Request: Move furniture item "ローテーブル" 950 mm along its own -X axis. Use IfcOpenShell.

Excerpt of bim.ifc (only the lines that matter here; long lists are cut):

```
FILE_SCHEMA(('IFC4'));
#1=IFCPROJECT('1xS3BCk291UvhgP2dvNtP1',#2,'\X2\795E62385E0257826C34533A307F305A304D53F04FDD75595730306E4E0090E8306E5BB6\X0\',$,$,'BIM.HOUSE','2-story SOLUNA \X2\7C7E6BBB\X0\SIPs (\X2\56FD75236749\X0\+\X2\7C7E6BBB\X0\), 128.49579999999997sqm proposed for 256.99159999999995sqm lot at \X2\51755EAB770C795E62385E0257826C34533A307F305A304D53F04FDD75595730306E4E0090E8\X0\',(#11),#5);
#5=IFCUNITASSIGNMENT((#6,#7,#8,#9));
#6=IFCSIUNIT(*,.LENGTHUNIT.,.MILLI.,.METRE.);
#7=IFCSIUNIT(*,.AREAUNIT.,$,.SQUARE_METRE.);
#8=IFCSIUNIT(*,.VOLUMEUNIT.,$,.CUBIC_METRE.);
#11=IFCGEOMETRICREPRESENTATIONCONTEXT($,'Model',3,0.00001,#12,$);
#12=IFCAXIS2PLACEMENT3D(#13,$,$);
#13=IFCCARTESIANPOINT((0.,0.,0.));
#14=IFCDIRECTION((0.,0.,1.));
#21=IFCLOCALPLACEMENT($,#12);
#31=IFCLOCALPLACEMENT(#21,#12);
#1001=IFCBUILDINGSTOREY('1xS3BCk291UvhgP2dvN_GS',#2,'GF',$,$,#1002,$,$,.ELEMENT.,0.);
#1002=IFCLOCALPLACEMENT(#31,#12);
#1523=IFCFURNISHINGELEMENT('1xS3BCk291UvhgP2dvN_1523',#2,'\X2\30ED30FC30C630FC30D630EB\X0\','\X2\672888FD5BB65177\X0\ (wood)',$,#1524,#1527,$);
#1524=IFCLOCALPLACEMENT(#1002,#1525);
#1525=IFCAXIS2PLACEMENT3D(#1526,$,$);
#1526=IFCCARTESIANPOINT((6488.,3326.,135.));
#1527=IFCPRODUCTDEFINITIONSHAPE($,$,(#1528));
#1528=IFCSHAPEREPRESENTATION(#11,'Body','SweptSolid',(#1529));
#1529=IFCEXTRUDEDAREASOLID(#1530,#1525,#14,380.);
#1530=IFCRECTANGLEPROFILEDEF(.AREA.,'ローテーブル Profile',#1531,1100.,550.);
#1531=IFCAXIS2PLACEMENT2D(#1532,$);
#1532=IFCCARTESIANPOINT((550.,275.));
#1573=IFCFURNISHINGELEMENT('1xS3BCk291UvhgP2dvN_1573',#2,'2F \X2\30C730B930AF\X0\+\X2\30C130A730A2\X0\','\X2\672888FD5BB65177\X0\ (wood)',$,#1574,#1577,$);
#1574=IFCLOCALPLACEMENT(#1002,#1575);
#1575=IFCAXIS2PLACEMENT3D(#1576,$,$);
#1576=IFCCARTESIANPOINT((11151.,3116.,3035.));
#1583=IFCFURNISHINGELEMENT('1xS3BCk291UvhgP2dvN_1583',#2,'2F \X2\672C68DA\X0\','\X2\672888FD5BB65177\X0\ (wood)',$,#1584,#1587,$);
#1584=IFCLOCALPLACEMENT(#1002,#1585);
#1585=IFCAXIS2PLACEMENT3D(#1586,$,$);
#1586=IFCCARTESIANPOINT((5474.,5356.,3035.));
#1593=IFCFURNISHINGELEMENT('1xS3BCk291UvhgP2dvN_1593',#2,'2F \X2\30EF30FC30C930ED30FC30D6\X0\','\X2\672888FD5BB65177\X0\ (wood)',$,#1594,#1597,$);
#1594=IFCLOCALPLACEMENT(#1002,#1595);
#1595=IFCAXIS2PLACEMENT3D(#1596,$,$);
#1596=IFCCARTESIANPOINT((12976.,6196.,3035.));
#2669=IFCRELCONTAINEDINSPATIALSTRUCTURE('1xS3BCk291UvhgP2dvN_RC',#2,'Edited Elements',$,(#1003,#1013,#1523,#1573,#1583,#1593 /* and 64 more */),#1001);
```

```python
import ifcopenshell
import ifcopenshell.api.geometry
import ifcopenshell.util.placement

model = ifcopenshell.open("bim.ifc")

item = model.by_guid("1xS3BCk291UvhgP2dvN_1523")
matrix = ifcopenshell.util.placement.get_local_placement(item.ObjectPlacement)
matrix[:3, 3] -= matrix[:3, 0] * 950.0
ifcopenshell.api.geometry.edit_object_placement(model, product=item, matrix=matrix, is_si=False)

print(ifcopenshell.util.placement.get_local_placement(item.ObjectPlacement).round(3) + 0.0)

model.write("bim_v2.ifc")
```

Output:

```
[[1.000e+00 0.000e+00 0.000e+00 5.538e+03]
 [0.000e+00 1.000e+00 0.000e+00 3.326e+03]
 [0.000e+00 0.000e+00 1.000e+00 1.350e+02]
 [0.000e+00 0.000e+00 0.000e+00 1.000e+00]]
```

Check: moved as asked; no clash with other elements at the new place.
